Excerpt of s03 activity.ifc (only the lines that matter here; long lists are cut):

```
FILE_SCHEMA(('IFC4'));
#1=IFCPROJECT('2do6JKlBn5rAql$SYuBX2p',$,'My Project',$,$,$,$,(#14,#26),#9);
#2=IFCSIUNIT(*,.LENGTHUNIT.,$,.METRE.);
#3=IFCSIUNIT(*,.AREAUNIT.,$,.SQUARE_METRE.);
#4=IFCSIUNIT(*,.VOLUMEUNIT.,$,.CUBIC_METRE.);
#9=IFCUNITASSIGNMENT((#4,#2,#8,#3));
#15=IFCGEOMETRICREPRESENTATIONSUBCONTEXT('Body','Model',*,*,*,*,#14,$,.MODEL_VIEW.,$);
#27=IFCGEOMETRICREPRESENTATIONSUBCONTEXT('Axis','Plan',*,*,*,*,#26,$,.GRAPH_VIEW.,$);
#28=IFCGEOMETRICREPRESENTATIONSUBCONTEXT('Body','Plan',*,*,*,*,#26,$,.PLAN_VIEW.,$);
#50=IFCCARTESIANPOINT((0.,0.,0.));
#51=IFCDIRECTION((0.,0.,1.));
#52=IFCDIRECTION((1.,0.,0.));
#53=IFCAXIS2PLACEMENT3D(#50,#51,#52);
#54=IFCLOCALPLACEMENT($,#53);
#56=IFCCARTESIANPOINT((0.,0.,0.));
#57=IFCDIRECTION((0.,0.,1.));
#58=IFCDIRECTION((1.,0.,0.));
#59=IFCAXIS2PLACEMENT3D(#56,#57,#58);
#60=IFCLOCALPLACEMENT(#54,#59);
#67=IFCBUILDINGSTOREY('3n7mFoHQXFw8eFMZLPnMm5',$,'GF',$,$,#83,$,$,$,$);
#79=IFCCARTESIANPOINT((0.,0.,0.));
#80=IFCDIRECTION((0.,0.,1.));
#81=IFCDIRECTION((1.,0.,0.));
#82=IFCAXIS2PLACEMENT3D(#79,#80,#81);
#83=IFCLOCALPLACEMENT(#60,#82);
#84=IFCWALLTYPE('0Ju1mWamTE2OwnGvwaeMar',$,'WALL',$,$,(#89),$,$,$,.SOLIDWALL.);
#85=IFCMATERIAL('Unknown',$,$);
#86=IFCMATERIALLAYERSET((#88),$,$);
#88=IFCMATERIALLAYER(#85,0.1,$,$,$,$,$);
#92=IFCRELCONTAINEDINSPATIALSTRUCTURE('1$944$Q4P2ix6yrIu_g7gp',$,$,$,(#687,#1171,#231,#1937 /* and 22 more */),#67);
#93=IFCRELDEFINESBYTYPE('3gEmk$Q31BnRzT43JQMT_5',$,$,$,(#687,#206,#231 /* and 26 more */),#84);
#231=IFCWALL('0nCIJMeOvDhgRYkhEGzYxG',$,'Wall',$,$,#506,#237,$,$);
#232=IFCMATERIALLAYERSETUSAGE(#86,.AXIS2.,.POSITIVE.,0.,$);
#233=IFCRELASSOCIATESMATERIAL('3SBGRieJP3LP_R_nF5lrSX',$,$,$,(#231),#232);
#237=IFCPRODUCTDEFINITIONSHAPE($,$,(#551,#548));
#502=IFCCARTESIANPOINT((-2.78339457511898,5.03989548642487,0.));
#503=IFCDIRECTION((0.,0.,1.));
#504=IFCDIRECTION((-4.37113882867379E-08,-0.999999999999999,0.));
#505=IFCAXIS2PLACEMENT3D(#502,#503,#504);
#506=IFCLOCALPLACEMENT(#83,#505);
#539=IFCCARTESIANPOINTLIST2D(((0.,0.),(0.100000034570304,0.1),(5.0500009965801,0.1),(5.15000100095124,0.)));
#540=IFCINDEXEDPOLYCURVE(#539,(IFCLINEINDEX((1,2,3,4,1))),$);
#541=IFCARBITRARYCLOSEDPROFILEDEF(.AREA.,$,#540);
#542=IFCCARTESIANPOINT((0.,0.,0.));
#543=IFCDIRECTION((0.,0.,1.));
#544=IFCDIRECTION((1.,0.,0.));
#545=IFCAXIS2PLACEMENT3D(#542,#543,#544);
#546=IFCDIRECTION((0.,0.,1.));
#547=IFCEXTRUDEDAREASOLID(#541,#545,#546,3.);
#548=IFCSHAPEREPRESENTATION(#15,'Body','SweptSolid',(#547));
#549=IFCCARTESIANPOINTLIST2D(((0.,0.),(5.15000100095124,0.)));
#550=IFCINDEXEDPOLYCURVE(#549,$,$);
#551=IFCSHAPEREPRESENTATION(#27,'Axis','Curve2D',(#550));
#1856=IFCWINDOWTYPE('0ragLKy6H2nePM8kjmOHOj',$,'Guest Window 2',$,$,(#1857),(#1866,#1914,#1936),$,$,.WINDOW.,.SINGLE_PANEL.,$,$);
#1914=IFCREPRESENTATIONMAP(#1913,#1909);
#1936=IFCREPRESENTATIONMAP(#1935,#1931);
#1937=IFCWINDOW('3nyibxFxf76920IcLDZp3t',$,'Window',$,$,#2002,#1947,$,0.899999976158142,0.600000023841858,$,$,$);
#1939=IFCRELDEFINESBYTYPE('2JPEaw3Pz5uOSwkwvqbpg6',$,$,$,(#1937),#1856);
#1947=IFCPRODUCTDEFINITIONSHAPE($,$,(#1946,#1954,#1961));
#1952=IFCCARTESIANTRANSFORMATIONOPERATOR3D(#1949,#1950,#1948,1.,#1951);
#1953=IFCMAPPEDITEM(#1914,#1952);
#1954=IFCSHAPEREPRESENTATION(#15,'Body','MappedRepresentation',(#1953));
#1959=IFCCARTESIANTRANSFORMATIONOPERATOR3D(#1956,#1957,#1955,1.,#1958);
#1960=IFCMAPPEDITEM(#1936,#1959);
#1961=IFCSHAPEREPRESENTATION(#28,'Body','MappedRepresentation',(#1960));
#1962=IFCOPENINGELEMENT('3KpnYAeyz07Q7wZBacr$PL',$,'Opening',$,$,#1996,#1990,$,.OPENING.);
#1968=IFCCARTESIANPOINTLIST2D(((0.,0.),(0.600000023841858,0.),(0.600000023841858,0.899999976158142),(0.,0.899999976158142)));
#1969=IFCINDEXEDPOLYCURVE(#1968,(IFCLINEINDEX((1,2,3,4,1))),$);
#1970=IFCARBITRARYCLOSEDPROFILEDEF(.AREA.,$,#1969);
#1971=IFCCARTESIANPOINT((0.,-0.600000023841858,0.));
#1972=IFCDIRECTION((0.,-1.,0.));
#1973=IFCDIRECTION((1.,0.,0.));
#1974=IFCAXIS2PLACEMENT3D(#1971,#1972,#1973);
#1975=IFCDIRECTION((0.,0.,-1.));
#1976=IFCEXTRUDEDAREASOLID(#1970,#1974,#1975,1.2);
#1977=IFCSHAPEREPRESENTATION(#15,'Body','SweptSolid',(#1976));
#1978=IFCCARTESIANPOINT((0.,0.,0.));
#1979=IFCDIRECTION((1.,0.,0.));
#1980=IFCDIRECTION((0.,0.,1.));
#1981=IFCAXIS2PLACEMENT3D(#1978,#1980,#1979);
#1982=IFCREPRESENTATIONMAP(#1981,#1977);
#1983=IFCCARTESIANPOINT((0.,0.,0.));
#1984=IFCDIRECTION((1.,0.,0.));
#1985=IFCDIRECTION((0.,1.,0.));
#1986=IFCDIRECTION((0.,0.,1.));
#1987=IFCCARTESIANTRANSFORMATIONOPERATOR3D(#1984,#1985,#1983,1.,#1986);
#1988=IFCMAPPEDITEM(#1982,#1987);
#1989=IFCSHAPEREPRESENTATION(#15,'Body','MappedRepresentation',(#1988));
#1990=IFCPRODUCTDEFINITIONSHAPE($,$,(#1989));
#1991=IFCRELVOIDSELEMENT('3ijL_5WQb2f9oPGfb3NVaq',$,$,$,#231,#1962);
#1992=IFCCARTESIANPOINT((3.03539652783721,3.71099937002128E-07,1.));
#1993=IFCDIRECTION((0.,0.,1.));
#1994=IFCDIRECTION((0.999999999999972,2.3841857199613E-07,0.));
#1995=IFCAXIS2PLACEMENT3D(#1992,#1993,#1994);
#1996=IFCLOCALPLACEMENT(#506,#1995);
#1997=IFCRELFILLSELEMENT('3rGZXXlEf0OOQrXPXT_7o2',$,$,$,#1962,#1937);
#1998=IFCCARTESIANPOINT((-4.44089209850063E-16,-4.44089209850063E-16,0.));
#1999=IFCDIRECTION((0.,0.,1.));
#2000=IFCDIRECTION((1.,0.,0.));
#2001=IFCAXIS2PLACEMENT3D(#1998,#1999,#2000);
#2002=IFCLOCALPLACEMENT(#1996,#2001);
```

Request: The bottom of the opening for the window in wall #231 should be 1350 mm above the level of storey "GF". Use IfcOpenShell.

```python
import numpy as np
import ifcopenshell
import ifcopenshell.api.geometry
import ifcopenshell.geom
import ifcopenshell.util.element
import ifcopenshell.util.placement
import ifcopenshell.util.shape
import ifcopenshell.util.unit

model = ifcopenshell.open("s03 activity.ifc")
unit_scale = ifcopenshell.util.unit.calculate_unit_scale(model)

window = model.by_guid("3nyibxFxf76920IcLDZp3t")
opening = window.FillsVoids[0].RelatingOpeningElement
storey = ifcopenshell.util.element.get_container(window, ifc_class="IfcBuildingStorey")
level = ifcopenshell.util.placement.get_local_placement(storey.ObjectPlacement)[2, 3]

# The opening's origin need not be at the sill, so measure its lowest point.
shape = ifcopenshell.geom.create_shape(ifcopenshell.geom.settings(), opening)
bottom = ifcopenshell.util.shape.get_shape_bottom_elevation(shape, shape.geometry) / unit_scale
dz = level + 1.35 - bottom

shift = np.array([0.0, 0.0, dz])
# The window is placed relative to its opening, so it follows when the opening moves.
matrix = ifcopenshell.util.placement.get_local_placement(opening.ObjectPlacement)
matrix[:3, 3] += shift
ifcopenshell.api.geometry.edit_object_placement(
    model, product=opening, matrix=matrix, is_si=False, should_transform_children=True
)

print(f"moved by {dz * unit_scale:+.3f} m")

model.write("s03 activity_rev.ifc")
```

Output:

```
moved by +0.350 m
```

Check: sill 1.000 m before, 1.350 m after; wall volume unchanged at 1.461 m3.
